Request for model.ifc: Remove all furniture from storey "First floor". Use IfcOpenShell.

First a look at what the model holds.

```python
import ifcopenshell
import ifcopenshell.util.element

model = ifcopenshell.open("model.ifc")
print(model.schema)
storey = next(s for s in model.by_type("IfcBuildingStorey") if s.Name == "First floor")
furniture = [e for e in ifcopenshell.util.element.get_decomposition(storey) if e.is_a("IfcFurnishingElement")]
seen = {}
for e in furniture:
    element_type = ifcopenshell.util.element.get_type(e)
    name = element_type.Name if element_type not in (None, e) else None
    seen[name] = seen.get(name, 0) + 1
for name, count in sorted(seen.items(), key=str):
    print(count, "x", name)
```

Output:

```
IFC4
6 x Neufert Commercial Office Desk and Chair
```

```python
import ifcopenshell
import ifcopenshell.api.root
import ifcopenshell.util.element

model = ifcopenshell.open("model.ifc")

storey = next(s for s in model.by_type("IfcBuildingStorey") if s.Name == "First floor")
furniture = [e for e in ifcopenshell.util.element.get_decomposition(storey) if e.is_a("IfcFurnishingElement")]

for e in furniture:
    ifcopenshell.api.root.remove_product(model, product=e)
print(len(furniture), "removed")

model.write("model_v2.ifc")
```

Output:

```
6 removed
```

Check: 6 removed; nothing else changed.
